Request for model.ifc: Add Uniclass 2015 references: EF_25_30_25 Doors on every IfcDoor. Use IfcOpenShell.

First a look at what the model holds.

```python
import ifcopenshell

model = ifcopenshell.open("model.ifc")
print(model.schema)
print("classifications:", [c.Name for c in model.by_type("IfcClassification")])
for ifc_class in ("IfcDoor", "IfcRoof", "IfcStair", "IfcWall", "IfcWindow"):
    print(ifc_class, len(model.by_type(ifc_class)))
```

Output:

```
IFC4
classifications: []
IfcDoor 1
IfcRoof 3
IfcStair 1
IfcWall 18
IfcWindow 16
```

```python
import ifcopenshell
import ifcopenshell.api.classification

model = ifcopenshell.open("model.ifc")

system = ifcopenshell.api.classification.add_classification(model, classification="Uniclass 2015")

codes = {
    "IfcDoor": ("EF_25_30_25", "Doors"),
}
for ifc_class, (code, name) in codes.items():
    products = model.by_type(ifc_class)
    ifcopenshell.api.classification.add_reference(
        model, products=products, classification=system, identification=code, name=name
    )
    print(code, len(products))

model.write("model_v2.ifc")
```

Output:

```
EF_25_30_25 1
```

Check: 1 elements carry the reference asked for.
